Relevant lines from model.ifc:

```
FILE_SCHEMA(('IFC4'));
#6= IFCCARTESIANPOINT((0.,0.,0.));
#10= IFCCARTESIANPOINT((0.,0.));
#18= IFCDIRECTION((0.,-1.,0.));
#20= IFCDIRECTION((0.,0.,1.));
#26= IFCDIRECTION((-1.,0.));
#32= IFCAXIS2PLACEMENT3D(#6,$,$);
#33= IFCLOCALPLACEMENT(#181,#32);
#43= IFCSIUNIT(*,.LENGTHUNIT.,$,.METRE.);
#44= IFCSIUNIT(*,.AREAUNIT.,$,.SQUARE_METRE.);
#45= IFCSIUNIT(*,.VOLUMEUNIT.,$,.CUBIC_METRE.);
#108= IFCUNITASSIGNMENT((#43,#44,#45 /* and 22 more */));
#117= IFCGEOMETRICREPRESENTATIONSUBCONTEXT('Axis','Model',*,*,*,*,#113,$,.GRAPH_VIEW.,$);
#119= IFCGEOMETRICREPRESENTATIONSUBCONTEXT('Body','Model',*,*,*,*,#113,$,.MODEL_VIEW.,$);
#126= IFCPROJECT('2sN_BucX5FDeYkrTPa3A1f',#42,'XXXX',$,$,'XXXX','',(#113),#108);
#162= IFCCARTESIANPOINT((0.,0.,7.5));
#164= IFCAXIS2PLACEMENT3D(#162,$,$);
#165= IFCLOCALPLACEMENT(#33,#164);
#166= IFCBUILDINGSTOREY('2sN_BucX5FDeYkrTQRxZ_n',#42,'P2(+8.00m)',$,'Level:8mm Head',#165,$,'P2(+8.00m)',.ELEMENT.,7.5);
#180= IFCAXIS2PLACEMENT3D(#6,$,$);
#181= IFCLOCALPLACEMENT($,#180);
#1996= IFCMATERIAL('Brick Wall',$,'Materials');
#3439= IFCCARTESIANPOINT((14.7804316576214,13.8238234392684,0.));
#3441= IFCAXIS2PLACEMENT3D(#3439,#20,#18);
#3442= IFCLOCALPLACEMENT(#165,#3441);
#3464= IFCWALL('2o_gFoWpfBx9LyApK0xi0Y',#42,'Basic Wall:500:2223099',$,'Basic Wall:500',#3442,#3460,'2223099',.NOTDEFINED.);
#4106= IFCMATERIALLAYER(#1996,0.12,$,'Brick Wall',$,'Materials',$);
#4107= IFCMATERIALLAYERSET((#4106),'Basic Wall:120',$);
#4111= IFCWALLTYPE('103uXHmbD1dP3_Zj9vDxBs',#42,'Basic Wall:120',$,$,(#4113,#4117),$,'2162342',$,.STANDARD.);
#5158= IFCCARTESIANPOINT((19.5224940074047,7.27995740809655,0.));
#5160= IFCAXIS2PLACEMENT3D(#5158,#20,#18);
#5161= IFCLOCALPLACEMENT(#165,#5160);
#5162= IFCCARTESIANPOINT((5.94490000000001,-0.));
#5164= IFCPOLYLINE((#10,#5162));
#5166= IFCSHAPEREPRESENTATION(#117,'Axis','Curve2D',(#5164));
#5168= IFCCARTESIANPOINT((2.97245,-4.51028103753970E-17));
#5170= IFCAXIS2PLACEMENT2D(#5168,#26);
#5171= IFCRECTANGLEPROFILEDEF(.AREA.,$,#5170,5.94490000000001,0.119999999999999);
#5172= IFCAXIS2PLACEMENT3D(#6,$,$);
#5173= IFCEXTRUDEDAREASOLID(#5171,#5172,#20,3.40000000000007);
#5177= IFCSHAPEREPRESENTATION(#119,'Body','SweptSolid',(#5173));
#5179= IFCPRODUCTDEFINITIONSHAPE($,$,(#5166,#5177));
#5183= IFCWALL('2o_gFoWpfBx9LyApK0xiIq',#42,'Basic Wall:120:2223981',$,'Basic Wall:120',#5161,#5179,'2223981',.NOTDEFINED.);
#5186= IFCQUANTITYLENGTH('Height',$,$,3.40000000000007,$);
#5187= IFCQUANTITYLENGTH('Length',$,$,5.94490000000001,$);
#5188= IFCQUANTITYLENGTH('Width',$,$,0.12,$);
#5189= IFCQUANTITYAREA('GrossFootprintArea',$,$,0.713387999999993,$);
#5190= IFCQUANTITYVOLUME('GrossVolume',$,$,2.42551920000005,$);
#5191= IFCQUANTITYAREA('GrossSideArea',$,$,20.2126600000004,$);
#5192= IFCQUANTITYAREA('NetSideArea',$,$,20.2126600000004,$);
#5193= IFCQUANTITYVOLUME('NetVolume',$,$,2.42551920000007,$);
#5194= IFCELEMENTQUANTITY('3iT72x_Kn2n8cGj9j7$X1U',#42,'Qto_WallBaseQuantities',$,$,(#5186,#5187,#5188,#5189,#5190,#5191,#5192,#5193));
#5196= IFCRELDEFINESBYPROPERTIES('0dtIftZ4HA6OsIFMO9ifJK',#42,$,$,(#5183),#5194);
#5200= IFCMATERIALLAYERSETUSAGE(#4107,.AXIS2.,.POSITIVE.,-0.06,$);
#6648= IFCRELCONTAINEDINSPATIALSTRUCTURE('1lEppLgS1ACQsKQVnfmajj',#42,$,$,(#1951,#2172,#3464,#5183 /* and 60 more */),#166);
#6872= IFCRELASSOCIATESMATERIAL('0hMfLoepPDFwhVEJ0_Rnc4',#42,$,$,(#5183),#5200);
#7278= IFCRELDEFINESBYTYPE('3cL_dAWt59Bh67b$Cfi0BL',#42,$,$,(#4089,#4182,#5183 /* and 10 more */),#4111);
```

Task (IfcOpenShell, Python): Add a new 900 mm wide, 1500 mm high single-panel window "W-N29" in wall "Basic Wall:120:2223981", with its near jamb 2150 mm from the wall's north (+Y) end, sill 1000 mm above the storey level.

```python
import numpy as np
import ifcopenshell
import ifcopenshell.api.feature
import ifcopenshell.api.geometry
import ifcopenshell.api.pset
import ifcopenshell.api.root
import ifcopenshell.api.spatial
import ifcopenshell.geom
import ifcopenshell.util.element
import ifcopenshell.util.placement
import ifcopenshell.util.representation
import ifcopenshell.util.shape
import ifcopenshell.util.unit

model = ifcopenshell.open("model.ifc")
unit_scale = ifcopenshell.util.unit.calculate_unit_scale(model)
area_scale = ifcopenshell.util.unit.calculate_unit_scale(model, "AREAUNIT")
volume_scale = ifcopenshell.util.unit.calculate_unit_scale(model, "VOLUMEUNIT")
settings = ifcopenshell.geom.settings()


def volume(element):
    """Net volume in cubic metres, openings subtracted."""
    shape = ifcopenshell.geom.create_shape(settings, element)
    return ifcopenshell.util.shape.get_volume(shape.geometry)


wall = model.by_id(5183)
storey = ifcopenshell.util.element.get_container(wall, ifc_class="IfcBuildingStorey")
context = ifcopenshell.util.representation.get_context(model, "Model", "Body", "MODEL_VIEW")
before = volume(wall)

width, height, from_end, sill = 0.9, 1.5, 2.15, 1  # metres

# The wall runs along its own X axis, and the end named is its -X end.
wall_shape = ifcopenshell.geom.create_shape(settings, wall)
x, y, z = ifcopenshell.util.shape.get_vertices(wall_shape.geometry).T
start = x.min() + from_end
face, thickness = float(y.min()), float(y.max() - y.min())
wall_matrix = ifcopenshell.util.placement.get_local_placement(wall.ObjectPlacement)
level = ifcopenshell.util.placement.get_local_placement(storey.ObjectPlacement)[2, 3]


def in_wall(x, y):
    """Placement at x, y metres in the wall's axes, at sill height."""
    matrix = wall_matrix.copy()
    matrix[:, 3] = wall_matrix @ np.array([x / unit_scale, y / unit_scale, 0.0, 1.0])
    matrix[2, 3] = level + sill / unit_scale
    return matrix


# Opening: a box that overshoots both wall faces by 50 mm.
opening = ifcopenshell.api.root.create_entity(model, ifc_class="IfcOpeningElement", predefined_type="OPENING")
box = ifcopenshell.api.geometry.add_wall_representation(
    model, context=context, length=width, height=height, thickness=thickness + 0.1
)
ifcopenshell.api.geometry.assign_representation(model, product=opening, representation=box)
ifcopenshell.api.geometry.edit_object_placement(model, product=opening, matrix=in_wall(start, face - 0.05), is_si=False)
ifcopenshell.api.feature.add_feature(model, feature=opening, element=wall)

window = ifcopenshell.api.root.create_entity(model, ifc_class="IfcWindow", name="W-N29", predefined_type="WINDOW")
window.OverallWidth, window.OverallHeight = width / unit_scale, height / unit_scale
window.PartitioningType = "SINGLE_PANEL"
body = ifcopenshell.api.geometry.add_window_representation(
    model,
    context=context,
    overall_width=window.OverallWidth,
    overall_height=window.OverallHeight,
    partition_type="SINGLE_PANEL",
)
ifcopenshell.api.geometry.assign_representation(model, product=window, representation=body)
ifcopenshell.api.spatial.assign_container(model, products=[window], relating_structure=storey)
ifcopenshell.api.feature.add_filling(model, opening=opening, element=window)

# Centre the window in the wall's thickness.
ifcopenshell.api.geometry.edit_object_placement(model, product=window, matrix=in_wall(start, face), is_si=False)
window_shape = ifcopenshell.geom.create_shape(settings, window)
depth = ifcopenshell.util.shape.get_vertices(window_shape.geometry)[:, 1]
offset = face + thickness / 2 - (depth.min() + depth.max()) / 2
ifcopenshell.api.geometry.edit_object_placement(model, product=window, matrix=in_wall(start, offset), is_si=False)

after = volume(wall)

# Update the wall's stored quantities.
qto = model.by_id(ifcopenshell.util.element.get_pset(wall, "Qto_WallBaseQuantities", should_inherit=False)["id"])
ifcopenshell.api.pset.edit_qto(model, qto=qto, properties={
    "NetSideArea": after / thickness / area_scale,
    "NetVolume": after / volume_scale,
})

print(f"wall volume {before:.3f} -> {after:.3f} m3")

model.write("model_updated.ifc")
```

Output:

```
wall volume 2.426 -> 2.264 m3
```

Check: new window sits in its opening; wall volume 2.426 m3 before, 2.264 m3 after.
